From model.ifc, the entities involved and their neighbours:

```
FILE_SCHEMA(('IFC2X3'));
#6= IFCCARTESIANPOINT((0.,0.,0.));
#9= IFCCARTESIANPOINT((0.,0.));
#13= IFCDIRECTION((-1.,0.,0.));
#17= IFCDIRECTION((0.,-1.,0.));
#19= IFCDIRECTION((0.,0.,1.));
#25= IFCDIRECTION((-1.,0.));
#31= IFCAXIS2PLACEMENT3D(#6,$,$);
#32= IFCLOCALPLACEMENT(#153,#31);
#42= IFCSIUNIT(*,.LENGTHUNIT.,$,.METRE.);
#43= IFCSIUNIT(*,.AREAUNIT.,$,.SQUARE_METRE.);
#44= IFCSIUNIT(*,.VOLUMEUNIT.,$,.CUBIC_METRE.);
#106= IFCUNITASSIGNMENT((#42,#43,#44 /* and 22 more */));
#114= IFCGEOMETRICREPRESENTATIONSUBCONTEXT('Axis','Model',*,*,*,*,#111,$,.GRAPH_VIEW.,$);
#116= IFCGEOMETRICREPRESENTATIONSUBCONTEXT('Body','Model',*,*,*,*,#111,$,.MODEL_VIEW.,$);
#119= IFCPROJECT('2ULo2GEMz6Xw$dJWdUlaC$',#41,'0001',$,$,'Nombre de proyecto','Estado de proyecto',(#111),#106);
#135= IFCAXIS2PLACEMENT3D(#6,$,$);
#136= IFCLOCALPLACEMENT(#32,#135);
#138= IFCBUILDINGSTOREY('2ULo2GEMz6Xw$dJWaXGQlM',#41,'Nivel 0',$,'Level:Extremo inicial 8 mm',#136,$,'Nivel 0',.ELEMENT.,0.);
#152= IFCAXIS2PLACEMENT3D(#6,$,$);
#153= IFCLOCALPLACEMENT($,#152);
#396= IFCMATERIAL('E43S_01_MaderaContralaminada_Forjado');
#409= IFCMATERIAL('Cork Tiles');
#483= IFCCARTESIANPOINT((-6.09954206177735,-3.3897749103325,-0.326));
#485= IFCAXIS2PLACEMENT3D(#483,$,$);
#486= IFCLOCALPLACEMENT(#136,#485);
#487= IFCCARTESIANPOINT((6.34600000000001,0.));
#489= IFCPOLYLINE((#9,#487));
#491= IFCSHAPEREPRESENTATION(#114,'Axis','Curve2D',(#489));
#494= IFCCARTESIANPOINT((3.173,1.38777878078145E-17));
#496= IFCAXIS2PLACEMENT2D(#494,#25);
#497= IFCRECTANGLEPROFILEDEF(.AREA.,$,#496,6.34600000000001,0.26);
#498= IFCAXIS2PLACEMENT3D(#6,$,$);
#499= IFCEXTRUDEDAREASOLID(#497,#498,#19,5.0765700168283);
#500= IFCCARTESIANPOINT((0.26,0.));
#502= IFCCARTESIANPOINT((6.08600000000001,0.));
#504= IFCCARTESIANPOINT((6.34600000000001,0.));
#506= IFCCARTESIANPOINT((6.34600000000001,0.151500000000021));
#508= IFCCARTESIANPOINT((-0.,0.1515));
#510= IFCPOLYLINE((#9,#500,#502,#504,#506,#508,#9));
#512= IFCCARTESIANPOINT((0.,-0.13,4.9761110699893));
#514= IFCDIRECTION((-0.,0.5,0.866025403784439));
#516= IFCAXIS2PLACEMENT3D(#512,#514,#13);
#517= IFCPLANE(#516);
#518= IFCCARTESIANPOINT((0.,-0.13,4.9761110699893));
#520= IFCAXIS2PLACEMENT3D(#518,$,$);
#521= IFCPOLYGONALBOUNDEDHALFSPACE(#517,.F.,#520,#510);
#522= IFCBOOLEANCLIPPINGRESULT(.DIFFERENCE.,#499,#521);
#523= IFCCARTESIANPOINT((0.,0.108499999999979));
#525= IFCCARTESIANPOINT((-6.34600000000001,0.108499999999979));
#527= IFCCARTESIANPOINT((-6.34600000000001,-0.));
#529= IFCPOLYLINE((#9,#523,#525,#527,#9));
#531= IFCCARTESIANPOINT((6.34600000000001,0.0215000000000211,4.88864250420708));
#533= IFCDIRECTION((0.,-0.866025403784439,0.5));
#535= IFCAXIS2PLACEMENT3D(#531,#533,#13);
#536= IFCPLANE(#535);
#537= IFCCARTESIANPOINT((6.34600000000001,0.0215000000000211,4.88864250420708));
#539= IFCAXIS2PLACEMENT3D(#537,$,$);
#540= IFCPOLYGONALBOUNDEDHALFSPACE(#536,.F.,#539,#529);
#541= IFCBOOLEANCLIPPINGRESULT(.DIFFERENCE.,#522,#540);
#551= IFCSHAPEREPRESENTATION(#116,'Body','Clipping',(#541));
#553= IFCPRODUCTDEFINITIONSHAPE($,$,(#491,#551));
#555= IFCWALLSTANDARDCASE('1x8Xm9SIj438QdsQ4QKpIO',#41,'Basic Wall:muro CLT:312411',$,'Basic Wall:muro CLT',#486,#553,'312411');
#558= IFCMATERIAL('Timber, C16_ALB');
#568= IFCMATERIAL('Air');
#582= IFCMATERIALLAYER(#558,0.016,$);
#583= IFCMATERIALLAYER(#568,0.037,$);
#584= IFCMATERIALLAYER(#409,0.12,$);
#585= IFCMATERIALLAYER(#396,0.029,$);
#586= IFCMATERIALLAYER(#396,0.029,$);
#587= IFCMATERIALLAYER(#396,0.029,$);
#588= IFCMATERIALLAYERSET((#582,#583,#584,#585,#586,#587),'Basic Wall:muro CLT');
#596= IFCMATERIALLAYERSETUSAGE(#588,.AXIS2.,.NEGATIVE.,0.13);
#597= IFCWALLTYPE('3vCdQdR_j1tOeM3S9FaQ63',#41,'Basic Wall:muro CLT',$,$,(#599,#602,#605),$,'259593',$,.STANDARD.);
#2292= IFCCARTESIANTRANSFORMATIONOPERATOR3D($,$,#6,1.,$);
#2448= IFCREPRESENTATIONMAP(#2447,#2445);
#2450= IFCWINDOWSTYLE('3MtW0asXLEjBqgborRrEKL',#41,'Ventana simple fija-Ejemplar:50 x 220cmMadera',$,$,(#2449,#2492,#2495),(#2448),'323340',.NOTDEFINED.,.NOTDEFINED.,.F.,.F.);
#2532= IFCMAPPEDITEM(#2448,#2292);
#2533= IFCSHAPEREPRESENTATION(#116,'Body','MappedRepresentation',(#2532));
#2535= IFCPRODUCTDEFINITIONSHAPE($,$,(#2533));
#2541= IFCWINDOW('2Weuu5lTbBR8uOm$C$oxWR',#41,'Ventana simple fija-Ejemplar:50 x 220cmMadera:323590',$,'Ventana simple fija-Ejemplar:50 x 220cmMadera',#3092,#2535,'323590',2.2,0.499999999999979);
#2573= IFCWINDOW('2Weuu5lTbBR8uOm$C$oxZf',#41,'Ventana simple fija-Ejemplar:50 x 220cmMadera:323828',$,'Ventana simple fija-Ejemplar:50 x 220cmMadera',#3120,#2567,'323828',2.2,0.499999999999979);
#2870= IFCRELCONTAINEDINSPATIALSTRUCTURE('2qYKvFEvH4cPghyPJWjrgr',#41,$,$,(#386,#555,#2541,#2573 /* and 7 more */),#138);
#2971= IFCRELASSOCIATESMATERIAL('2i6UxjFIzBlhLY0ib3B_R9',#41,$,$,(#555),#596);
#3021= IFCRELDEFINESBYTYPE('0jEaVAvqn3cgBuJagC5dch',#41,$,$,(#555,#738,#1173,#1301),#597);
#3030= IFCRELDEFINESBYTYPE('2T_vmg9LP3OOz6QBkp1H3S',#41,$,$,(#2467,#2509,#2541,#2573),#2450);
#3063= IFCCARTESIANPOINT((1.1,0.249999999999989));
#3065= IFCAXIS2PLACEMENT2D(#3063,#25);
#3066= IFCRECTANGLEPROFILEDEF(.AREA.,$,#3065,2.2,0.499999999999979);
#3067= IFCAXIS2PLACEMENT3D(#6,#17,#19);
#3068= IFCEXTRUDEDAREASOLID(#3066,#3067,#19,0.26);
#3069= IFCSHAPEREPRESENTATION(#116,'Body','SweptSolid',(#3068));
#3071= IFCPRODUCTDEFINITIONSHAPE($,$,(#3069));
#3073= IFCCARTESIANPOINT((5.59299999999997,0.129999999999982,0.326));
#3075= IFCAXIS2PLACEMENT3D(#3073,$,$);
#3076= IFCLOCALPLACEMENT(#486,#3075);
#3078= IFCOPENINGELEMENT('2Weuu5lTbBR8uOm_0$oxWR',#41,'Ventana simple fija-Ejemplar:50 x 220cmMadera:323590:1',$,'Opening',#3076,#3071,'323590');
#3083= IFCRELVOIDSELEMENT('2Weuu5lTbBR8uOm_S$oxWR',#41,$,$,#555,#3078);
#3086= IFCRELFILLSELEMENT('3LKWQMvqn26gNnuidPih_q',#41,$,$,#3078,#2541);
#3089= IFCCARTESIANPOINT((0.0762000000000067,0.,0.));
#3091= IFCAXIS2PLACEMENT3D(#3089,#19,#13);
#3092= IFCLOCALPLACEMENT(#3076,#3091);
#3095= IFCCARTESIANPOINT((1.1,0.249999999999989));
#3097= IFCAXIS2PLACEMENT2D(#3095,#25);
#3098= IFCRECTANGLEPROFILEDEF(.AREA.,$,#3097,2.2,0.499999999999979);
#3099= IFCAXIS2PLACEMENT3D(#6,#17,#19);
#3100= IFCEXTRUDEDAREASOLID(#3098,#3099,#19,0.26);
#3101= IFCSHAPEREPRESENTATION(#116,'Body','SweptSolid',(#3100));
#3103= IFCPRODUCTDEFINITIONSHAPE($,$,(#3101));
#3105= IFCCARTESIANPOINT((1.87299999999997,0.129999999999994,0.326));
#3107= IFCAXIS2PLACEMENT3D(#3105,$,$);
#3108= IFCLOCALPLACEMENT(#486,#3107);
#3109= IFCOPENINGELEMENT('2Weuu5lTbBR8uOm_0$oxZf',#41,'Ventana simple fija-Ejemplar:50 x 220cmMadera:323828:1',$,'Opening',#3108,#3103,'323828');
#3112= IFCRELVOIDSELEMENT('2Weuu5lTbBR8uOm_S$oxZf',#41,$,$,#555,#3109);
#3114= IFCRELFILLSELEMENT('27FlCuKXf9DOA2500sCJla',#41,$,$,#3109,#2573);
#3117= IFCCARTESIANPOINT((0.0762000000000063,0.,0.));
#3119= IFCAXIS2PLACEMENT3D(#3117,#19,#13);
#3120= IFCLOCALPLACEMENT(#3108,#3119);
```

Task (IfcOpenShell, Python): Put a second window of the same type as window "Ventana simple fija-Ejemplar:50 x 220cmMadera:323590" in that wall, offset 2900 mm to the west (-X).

```python
import ifcopenshell
import ifcopenshell.api.feature
import ifcopenshell.api.geometry
import ifcopenshell.api.root
import ifcopenshell.geom
import ifcopenshell.util.element
import ifcopenshell.util.placement
import ifcopenshell.util.shape
import ifcopenshell.util.unit

model = ifcopenshell.open("model.ifc")
unit_scale = ifcopenshell.util.unit.calculate_unit_scale(model)
settings = ifcopenshell.geom.settings()


def volume(element):
    """Net volume in cubic metres, openings subtracted."""
    shape = ifcopenshell.geom.create_shape(settings, element)
    return ifcopenshell.util.shape.get_volume(shape.geometry)


def reuse_history(source, copy):
    """copy_class also copies each property set's owner history, people and application; keep the originals."""
    for rel in copy.IsDefinedBy:
        if rel.is_a("IfcRelDefinesByProperties") and (history := rel.RelatingPropertyDefinition.OwnerHistory):
            rel.RelatingPropertyDefinition.OwnerHistory = source.OwnerHistory
            ifcopenshell.util.element.remove_deep2(model, history)


window = model.by_id(2541)
opening = window.FillsVoids[0].RelatingOpeningElement
wall = opening.VoidsElements[0].RelatingBuildingElement
before = volume(wall)
shift = ifcopenshell.util.placement.get_local_placement(wall.ObjectPlacement)[:3, 0] * -2.9 / unit_scale

# copy_class copies the void relationship, type, container and properties, but no geometry.
new_opening = ifcopenshell.api.root.copy_class(model, product=opening)
new_opening.Representation = ifcopenshell.util.element.copy_deep(
    model, opening.Representation, exclude=["IfcGeometricRepresentationContext", "IfcRepresentationMap"]
)
new_opening.Name = "Ventana simple fija-Ejemplar:50 x 220cmMadera"
new_opening.Tag = None
new_window = ifcopenshell.api.root.copy_class(model, product=window)
new_window.Representation = ifcopenshell.util.element.copy_deep(
    model, window.Representation, exclude=["IfcGeometricRepresentationContext", "IfcRepresentationMap"]
)
new_window.Name = "Ventana simple fija-Ejemplar:50 x 220cmMadera"
new_window.Tag = None
reuse_history(window, new_window)
fills = ifcopenshell.api.feature.add_filling(model, opening=new_opening, element=new_window)
fills.OwnerHistory = new_window.OwnerHistory  # required in IFC2X3

for old, new in ((opening, new_opening), (window, new_window)):
    matrix = ifcopenshell.util.placement.get_local_placement(old.ObjectPlacement)
    matrix[:3, 3] += shift
    ifcopenshell.api.geometry.edit_object_placement(model, product=new, matrix=matrix, is_si=False)

after = volume(wall)

print(f"wall volume {before:.3f} -> {after:.3f} m3")

model.write("model_v2.ifc")
```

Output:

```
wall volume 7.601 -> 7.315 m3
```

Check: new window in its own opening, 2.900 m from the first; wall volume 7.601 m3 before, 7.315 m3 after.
